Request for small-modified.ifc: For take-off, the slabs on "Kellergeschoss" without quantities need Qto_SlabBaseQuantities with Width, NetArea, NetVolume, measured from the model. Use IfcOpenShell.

First a look at what the model holds.

```python
import ifcopenshell
import ifcopenshell.util.element
import ifcopenshell.util.unit

model = ifcopenshell.open("small-modified.ifc")
print(model.schema)
for unit_type in ("LENGTHUNIT", "AREAUNIT", "VOLUMEUNIT"):
    print(unit_type, ifcopenshell.util.unit.calculate_unit_scale(model, unit_type))
storey = next(s for s in model.by_type("IfcBuildingStorey") if s.Name == "Kellergeschoss")
slabs = [e for e in ifcopenshell.util.element.get_decomposition(storey) if e.is_a("IfcSlab")]
for e in sorted(slabs, key=lambda e: e.id()):
    print(e.id(), e.is_a(), e.Name, list(ifcopenshell.util.element.get_psets(e, qtos_only=True)), sep=" | ")
```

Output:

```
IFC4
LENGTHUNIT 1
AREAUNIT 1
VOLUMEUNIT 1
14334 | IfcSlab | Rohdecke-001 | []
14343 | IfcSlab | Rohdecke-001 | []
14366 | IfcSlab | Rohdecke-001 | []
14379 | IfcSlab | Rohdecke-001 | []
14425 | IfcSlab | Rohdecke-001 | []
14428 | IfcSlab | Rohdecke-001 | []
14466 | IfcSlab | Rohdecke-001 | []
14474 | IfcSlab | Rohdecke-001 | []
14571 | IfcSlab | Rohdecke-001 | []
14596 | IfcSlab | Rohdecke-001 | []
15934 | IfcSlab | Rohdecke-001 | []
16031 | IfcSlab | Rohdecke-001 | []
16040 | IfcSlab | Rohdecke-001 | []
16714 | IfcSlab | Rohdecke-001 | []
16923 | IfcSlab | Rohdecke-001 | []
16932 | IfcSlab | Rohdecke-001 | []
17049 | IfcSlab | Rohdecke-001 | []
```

```python
import ifcopenshell
import ifcopenshell.api.pset
import ifcopenshell.geom
import ifcopenshell.util.element
import ifcopenshell.util.shape
import ifcopenshell.util.unit

model = ifcopenshell.open("small-modified.ifc")
unit_scale = ifcopenshell.util.unit.calculate_unit_scale(model)
area_scale = ifcopenshell.util.unit.calculate_unit_scale(model, "AREAUNIT")
volume_scale = ifcopenshell.util.unit.calculate_unit_scale(model, "VOLUMEUNIT")
settings = ifcopenshell.geom.settings()

storey = next(s for s in model.by_type("IfcBuildingStorey") if s.Name == "Kellergeschoss")
slabs = [e for e in ifcopenshell.util.element.get_decomposition(storey) if e.is_a("IfcSlab")]

for e in sorted(slabs, key=lambda e: e.id()):
    if ifcopenshell.util.element.get_psets(e, qtos_only=True, should_inherit=False):
        continue
    # Geometry comes back in metres, in the element's own axes.
    shape = ifcopenshell.geom.create_shape(settings, e)
    values = {
        "Width": ifcopenshell.util.shape.get_z(shape.geometry) / unit_scale,
        "NetArea": ifcopenshell.util.shape.get_footprint_area(shape.geometry) / area_scale,
        "NetVolume": ifcopenshell.util.shape.get_volume(shape.geometry) / volume_scale,
    }
    qto = ifcopenshell.api.pset.add_qto(model, product=e, name="Qto_SlabBaseQuantities")
    ifcopenshell.api.pset.edit_qto(model, qto=qto, properties=values)
    print(e.id(), {k: round(v, 3) for k, v in values.items()})

model.write("small-modified_rev.ifc")
```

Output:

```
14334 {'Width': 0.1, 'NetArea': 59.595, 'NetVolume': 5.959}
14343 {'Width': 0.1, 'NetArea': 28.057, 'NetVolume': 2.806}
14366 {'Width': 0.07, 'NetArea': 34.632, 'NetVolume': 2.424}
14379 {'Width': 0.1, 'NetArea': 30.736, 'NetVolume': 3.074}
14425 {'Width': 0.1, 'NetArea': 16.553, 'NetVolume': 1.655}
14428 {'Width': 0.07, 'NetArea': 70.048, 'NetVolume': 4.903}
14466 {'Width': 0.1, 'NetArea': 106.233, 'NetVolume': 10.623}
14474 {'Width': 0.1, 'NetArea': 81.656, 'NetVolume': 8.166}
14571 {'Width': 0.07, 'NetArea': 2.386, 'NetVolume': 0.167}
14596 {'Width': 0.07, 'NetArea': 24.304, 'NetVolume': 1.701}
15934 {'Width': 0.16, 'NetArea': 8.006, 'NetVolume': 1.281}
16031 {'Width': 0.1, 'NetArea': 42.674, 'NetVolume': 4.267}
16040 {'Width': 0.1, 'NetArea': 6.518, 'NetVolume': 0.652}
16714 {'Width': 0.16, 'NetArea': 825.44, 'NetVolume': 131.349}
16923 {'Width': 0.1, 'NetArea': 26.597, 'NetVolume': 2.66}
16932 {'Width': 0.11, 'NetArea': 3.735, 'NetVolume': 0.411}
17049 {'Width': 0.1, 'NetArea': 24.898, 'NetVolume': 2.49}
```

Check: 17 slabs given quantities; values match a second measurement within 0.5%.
